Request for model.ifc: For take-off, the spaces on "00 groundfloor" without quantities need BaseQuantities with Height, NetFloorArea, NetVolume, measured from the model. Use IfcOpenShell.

First a look at what the model holds.

```python
import ifcopenshell
import ifcopenshell.util.element
import ifcopenshell.util.unit

model = ifcopenshell.open("model.ifc")
print(model.schema)
for unit_type in ("LENGTHUNIT", "AREAUNIT", "VOLUMEUNIT"):
    print(unit_type, ifcopenshell.util.unit.calculate_unit_scale(model, unit_type))
storey = next(s for s in model.by_type("IfcBuildingStorey") if s.Name == "00 groundfloor")
spaces = [e for e in ifcopenshell.util.element.get_decomposition(storey) if e.is_a("IfcSpace")]
for e in sorted(spaces, key=lambda e: e.id()):
    print(e.id(), e.is_a(), e.Name, list(ifcopenshell.util.element.get_psets(e, qtos_only=True)), sep=" | ")
```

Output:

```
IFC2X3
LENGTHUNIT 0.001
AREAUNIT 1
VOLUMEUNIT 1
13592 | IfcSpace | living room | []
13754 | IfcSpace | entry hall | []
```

```python
import ifcopenshell
import ifcopenshell.api.pset
import ifcopenshell.geom
import ifcopenshell.util.element
import ifcopenshell.util.shape
import ifcopenshell.util.unit

model = ifcopenshell.open("model.ifc")
unit_scale = ifcopenshell.util.unit.calculate_unit_scale(model)
area_scale = ifcopenshell.util.unit.calculate_unit_scale(model, "AREAUNIT")
volume_scale = ifcopenshell.util.unit.calculate_unit_scale(model, "VOLUMEUNIT")
settings = ifcopenshell.geom.settings()

storey = next(s for s in model.by_type("IfcBuildingStorey") if s.Name == "00 groundfloor")
spaces = [e for e in ifcopenshell.util.element.get_decomposition(storey) if e.is_a("IfcSpace")]

for e in sorted(spaces, key=lambda e: e.id()):
    if ifcopenshell.util.element.get_psets(e, qtos_only=True, should_inherit=False):
        continue
    # Geometry comes back in metres, in the element's own axes.
    shape = ifcopenshell.geom.create_shape(settings, e)
    values = {
        "Height": ifcopenshell.util.shape.get_z(shape.geometry) / unit_scale,
        "NetFloorArea": ifcopenshell.util.shape.get_footprint_area(shape.geometry) / area_scale,
        "NetVolume": ifcopenshell.util.shape.get_volume(shape.geometry) / volume_scale,
    }
    qto = ifcopenshell.api.pset.add_qto(model, product=e, name="BaseQuantities")
    ifcopenshell.api.pset.edit_qto(model, qto=qto, properties=values)
    print(e.id(), {k: round(v, 3) for k, v in values.items()})

model.write("model-out.ifc")
```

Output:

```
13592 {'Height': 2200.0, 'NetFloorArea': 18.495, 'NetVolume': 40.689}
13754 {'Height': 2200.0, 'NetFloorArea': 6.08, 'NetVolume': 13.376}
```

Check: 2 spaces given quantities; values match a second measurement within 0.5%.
